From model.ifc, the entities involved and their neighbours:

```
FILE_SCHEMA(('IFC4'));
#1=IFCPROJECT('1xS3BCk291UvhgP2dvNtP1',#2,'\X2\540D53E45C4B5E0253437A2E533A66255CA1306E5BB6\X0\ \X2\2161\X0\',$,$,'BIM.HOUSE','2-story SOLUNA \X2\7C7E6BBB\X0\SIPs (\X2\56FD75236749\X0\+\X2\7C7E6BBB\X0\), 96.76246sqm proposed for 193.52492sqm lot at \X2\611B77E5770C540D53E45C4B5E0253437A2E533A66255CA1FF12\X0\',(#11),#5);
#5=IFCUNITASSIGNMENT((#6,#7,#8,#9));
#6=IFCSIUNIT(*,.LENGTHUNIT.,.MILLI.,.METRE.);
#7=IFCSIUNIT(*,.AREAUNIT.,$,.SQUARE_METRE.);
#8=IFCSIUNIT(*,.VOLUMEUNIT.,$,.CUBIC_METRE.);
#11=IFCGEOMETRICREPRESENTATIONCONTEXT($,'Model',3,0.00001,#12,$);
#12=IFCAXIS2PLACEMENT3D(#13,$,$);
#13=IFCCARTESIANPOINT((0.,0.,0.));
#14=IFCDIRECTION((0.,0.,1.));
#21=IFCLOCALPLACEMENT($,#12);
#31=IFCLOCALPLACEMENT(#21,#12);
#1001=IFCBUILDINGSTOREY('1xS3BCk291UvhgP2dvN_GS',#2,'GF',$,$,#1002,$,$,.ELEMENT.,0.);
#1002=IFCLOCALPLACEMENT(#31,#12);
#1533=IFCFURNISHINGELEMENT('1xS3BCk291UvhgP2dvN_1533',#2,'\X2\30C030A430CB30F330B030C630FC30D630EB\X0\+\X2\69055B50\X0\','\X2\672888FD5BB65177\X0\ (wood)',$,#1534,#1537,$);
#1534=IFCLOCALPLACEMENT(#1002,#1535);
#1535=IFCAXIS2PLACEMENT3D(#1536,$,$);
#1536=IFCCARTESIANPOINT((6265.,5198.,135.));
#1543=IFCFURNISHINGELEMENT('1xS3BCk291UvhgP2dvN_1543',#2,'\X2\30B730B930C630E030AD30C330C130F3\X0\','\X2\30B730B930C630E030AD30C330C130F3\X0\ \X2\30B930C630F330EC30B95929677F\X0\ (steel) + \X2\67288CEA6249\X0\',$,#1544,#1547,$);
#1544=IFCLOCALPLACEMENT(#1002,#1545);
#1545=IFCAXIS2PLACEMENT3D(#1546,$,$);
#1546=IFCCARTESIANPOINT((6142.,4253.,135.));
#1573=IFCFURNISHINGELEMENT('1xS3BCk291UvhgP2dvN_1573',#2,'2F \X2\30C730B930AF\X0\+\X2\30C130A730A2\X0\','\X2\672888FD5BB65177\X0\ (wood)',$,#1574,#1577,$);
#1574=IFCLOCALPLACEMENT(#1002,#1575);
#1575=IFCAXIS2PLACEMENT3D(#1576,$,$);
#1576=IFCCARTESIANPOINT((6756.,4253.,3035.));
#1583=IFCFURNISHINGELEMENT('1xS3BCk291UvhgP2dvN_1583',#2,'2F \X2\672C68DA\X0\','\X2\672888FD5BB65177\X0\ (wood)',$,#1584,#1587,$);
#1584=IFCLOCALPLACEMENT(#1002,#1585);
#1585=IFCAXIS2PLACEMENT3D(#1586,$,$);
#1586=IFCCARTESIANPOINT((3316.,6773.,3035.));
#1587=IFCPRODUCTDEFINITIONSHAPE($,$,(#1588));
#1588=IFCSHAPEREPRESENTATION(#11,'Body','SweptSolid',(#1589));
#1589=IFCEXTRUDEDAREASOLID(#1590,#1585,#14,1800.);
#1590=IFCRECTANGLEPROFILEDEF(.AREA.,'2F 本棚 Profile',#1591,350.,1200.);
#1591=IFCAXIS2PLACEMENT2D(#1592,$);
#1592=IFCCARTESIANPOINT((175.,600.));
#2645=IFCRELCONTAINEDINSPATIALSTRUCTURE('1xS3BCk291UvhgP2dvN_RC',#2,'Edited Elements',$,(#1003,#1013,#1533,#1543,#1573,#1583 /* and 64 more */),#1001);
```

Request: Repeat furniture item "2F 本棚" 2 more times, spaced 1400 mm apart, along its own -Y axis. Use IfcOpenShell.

```python
import ifcopenshell
import ifcopenshell.api.geometry
import ifcopenshell.api.root
import ifcopenshell.util.element
import ifcopenshell.util.placement
import ifcopenshell.util.unit

model = ifcopenshell.open("model.ifc")
unit_scale = ifcopenshell.util.unit.calculate_unit_scale(model)


def reuse_history(source, copy):
    """copy_class also copies each property set's owner history, people and application; keep the originals."""
    for rel in copy.IsDefinedBy:
        if rel.is_a("IfcRelDefinesByProperties") and (history := rel.RelatingPropertyDefinition.OwnerHistory):
            rel.RelatingPropertyDefinition.OwnerHistory = source.OwnerHistory
            ifcopenshell.util.element.remove_deep2(model, history)


source = model.by_guid("1xS3BCk291UvhgP2dvN_1583")
base = ifcopenshell.util.placement.get_local_placement(source.ObjectPlacement)
step = -base[:3, 1] * 1.4 / unit_scale

for i in range(1, 3):
    copy = ifcopenshell.api.root.copy_class(model, product=source)
    copy.Representation = ifcopenshell.util.element.copy_deep(
        model, source.Representation, exclude=["IfcGeometricRepresentationContext", "IfcRepresentationMap"]
    )
    reuse_history(source, copy)
    matrix = base.copy()
    matrix[:3, 3] += i * step
    print("added at", matrix[:3, 3].round(3) + 0.0)
    ifcopenshell.api.geometry.edit_object_placement(model, product=copy, matrix=matrix, is_si=False)

model.write("model_edited.ifc")
```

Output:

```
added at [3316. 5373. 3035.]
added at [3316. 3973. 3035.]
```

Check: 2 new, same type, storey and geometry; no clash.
